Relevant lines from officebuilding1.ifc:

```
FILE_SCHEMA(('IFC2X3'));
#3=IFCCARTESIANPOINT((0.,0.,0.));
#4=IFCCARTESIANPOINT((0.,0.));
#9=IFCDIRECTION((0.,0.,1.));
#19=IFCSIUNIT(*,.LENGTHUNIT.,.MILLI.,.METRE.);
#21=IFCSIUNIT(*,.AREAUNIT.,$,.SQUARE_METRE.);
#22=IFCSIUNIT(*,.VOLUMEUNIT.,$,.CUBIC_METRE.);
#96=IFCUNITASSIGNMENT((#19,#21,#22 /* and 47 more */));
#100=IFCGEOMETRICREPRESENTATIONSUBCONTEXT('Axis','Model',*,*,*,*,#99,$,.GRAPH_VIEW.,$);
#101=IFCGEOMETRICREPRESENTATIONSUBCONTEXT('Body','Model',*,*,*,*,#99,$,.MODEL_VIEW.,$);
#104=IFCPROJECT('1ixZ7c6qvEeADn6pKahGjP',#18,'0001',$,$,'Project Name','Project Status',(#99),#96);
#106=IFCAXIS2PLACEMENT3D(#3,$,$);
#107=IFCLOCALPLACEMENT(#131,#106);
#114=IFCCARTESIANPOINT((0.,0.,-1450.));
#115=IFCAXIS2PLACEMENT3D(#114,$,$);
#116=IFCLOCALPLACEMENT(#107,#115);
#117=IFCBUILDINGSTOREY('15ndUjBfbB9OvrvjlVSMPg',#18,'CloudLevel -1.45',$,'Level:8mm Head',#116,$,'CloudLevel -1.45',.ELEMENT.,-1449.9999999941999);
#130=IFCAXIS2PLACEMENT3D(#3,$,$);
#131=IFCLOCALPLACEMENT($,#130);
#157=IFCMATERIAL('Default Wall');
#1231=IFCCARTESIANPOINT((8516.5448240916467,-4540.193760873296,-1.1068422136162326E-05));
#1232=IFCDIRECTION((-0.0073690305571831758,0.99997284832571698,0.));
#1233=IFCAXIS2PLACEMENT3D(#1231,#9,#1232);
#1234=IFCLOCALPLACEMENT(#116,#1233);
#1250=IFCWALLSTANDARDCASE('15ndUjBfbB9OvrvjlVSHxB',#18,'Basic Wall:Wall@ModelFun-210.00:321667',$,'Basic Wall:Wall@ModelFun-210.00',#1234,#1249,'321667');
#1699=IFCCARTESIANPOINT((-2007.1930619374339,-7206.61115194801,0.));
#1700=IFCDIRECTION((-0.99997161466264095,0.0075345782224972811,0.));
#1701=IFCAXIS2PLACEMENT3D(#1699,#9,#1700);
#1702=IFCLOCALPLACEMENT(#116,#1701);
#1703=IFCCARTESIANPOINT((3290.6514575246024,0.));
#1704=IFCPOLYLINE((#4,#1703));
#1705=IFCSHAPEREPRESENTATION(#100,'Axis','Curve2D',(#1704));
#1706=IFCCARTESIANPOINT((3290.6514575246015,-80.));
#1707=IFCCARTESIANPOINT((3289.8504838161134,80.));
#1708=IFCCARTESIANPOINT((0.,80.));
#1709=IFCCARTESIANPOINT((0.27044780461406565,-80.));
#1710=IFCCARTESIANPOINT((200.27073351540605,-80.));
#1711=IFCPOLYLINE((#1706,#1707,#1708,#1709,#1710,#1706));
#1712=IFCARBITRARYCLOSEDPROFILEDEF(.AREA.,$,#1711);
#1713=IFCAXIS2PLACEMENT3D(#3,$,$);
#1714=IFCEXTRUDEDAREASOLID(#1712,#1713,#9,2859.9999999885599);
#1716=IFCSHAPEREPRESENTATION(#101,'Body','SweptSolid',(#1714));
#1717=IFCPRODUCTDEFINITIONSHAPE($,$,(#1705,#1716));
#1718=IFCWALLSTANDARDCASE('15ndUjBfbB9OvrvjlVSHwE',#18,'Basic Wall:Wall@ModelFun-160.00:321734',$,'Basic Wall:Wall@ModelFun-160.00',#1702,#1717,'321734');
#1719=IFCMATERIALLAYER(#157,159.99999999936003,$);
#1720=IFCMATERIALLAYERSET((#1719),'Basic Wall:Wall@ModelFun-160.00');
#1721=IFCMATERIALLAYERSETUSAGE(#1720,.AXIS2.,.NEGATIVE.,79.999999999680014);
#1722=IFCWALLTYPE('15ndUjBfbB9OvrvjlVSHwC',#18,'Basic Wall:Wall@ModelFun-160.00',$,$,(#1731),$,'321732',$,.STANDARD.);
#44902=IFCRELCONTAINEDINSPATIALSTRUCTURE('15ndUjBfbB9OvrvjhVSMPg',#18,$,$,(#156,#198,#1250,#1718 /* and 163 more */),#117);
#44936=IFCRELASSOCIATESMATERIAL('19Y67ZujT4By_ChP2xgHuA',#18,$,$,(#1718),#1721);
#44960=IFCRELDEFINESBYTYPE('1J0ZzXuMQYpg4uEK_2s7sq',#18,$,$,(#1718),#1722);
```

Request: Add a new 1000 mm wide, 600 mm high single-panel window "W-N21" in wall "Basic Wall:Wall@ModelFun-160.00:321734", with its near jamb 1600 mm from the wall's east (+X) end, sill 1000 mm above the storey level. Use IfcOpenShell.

```python
import numpy as np
import ifcopenshell
import ifcopenshell.api.feature
import ifcopenshell.api.geometry
import ifcopenshell.api.root
import ifcopenshell.api.spatial
import ifcopenshell.api.type
import ifcopenshell.geom
import ifcopenshell.util.element
import ifcopenshell.util.placement
import ifcopenshell.util.representation
import ifcopenshell.util.shape
import ifcopenshell.util.unit

model = ifcopenshell.open("officebuilding1.ifc")
unit_scale = ifcopenshell.util.unit.calculate_unit_scale(model)
settings = ifcopenshell.geom.settings()


def volume(element):
    """Net volume in cubic metres, openings subtracted."""
    shape = ifcopenshell.geom.create_shape(settings, element)
    return ifcopenshell.util.shape.get_volume(shape.geometry)


wall = model.by_id(1718)
storey = ifcopenshell.util.element.get_container(wall, ifc_class="IfcBuildingStorey")
context = ifcopenshell.util.representation.get_context(model, "Model", "Body", "MODEL_VIEW")
before = volume(wall)

width, height, from_end, sill = 1, 0.6, 1.6, 1  # metres

# The wall runs along its own X axis, and the end named is its -X end.
wall_shape = ifcopenshell.geom.create_shape(settings, wall)
x, y, z = ifcopenshell.util.shape.get_vertices(wall_shape.geometry).T
start = x.min() + from_end
face, thickness = float(y.min()), float(y.max() - y.min())
wall_matrix = ifcopenshell.util.placement.get_local_placement(wall.ObjectPlacement)
level = ifcopenshell.util.placement.get_local_placement(storey.ObjectPlacement)[2, 3]


def in_wall(x, y):
    """Placement at x, y metres in the wall's axes, at sill height."""
    matrix = wall_matrix.copy()
    matrix[:, 3] = wall_matrix @ np.array([x / unit_scale, y / unit_scale, 0.0, 1.0])
    matrix[2, 3] = level + sill / unit_scale
    return matrix


# Opening: a box that overshoots both wall faces by 50 mm.
opening = ifcopenshell.api.root.create_entity(model, ifc_class="IfcOpeningElement")
box = ifcopenshell.api.geometry.add_wall_representation(
    model, context=context, length=width, height=height, thickness=thickness + 0.1
)
ifcopenshell.api.geometry.assign_representation(model, product=opening, representation=box)
ifcopenshell.api.geometry.edit_object_placement(model, product=opening, matrix=in_wall(start, face - 0.05), is_si=False)
ifcopenshell.api.feature.add_feature(model, feature=opening, element=wall)

window = ifcopenshell.api.root.create_entity(model, ifc_class="IfcWindow", name="W-N21")
window.OverallWidth, window.OverallHeight = width / unit_scale, height / unit_scale
body = ifcopenshell.api.geometry.add_window_representation(
    model,
    context=context,
    overall_width=window.OverallWidth,
    overall_height=window.OverallHeight,
    partition_type="SINGLE_PANEL",
)
ifcopenshell.api.geometry.assign_representation(model, product=window, representation=body)
ifcopenshell.api.spatial.assign_container(model, products=[window], relating_structure=storey)
fills = ifcopenshell.api.feature.add_filling(model, opening=opening, element=window)
fills.OwnerHistory = window.OwnerHistory  # required in IFC2X3

# IFC2X3 keeps the operation on the window style.
style = ifcopenshell.api.root.create_entity(model, ifc_class="IfcWindowStyle", name="W-N21")
style.OperationType, style.ConstructionType = "SINGLE_PANEL", "NOTDEFINED"
style.ParameterTakesPrecedence = style.Sizeable = False
ifcopenshell.api.type.assign_type(model, related_objects=[window], relating_type=style)

# Centre the window in the wall's thickness.
ifcopenshell.api.geometry.edit_object_placement(model, product=window, matrix=in_wall(start, face), is_si=False)
window_shape = ifcopenshell.geom.create_shape(settings, window)
depth = ifcopenshell.util.shape.get_vertices(window_shape.geometry)[:, 1]
offset = face + thickness / 2 - (depth.min() + depth.max()) / 2
ifcopenshell.api.geometry.edit_object_placement(model, product=window, matrix=in_wall(start, offset), is_si=False)

after = volume(wall)

print(f"wall volume {before:.3f} -> {after:.3f} m3")

model.write("officebuilding1_rev.ifc")
```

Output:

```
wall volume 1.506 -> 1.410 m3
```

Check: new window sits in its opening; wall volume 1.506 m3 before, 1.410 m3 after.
